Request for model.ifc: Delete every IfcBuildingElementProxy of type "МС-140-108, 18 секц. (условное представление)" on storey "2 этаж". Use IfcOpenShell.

First a look at what the model holds.

```python
import ifcopenshell
import ifcopenshell.util.element

model = ifcopenshell.open("model.ifc")
print(model.schema)
storey = next(s for s in model.by_type("IfcBuildingStorey") if s.Name == "2 этаж")
proxies = [e for e in ifcopenshell.util.element.get_decomposition(storey) if e.is_a("IfcBuildingElementProxy")]
seen = {}
for e in proxies:
    element_type = ifcopenshell.util.element.get_type(e)
    name = element_type.Name if element_type not in (None, e) else None
    seen[name] = seen.get(name, 0) + 1
for name, count in sorted(seen.items(), key=str):
    print(count, "x", name)
```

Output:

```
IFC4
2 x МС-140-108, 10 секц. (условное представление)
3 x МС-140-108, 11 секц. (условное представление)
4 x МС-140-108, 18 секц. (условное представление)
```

```python
import ifcopenshell
import ifcopenshell.api.root
import ifcopenshell.util.element

model = ifcopenshell.open("model.ifc")

storey = next(s for s in model.by_type("IfcBuildingStorey") if s.Name == "2 этаж")
proxies = [e for e in ifcopenshell.util.element.get_decomposition(storey) if e.is_a("IfcBuildingElementProxy")]
targets = [e for e in proxies if (t := ifcopenshell.util.element.get_type(e)) not in (None, e) and t.Name == "МС-140-108, 18 секц. (условное представление)"]

for e in targets:
    ifcopenshell.api.root.remove_product(model, product=e)
print(len(targets), "removed")

model.write("model_edited.ifc")
```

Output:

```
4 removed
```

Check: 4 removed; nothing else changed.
